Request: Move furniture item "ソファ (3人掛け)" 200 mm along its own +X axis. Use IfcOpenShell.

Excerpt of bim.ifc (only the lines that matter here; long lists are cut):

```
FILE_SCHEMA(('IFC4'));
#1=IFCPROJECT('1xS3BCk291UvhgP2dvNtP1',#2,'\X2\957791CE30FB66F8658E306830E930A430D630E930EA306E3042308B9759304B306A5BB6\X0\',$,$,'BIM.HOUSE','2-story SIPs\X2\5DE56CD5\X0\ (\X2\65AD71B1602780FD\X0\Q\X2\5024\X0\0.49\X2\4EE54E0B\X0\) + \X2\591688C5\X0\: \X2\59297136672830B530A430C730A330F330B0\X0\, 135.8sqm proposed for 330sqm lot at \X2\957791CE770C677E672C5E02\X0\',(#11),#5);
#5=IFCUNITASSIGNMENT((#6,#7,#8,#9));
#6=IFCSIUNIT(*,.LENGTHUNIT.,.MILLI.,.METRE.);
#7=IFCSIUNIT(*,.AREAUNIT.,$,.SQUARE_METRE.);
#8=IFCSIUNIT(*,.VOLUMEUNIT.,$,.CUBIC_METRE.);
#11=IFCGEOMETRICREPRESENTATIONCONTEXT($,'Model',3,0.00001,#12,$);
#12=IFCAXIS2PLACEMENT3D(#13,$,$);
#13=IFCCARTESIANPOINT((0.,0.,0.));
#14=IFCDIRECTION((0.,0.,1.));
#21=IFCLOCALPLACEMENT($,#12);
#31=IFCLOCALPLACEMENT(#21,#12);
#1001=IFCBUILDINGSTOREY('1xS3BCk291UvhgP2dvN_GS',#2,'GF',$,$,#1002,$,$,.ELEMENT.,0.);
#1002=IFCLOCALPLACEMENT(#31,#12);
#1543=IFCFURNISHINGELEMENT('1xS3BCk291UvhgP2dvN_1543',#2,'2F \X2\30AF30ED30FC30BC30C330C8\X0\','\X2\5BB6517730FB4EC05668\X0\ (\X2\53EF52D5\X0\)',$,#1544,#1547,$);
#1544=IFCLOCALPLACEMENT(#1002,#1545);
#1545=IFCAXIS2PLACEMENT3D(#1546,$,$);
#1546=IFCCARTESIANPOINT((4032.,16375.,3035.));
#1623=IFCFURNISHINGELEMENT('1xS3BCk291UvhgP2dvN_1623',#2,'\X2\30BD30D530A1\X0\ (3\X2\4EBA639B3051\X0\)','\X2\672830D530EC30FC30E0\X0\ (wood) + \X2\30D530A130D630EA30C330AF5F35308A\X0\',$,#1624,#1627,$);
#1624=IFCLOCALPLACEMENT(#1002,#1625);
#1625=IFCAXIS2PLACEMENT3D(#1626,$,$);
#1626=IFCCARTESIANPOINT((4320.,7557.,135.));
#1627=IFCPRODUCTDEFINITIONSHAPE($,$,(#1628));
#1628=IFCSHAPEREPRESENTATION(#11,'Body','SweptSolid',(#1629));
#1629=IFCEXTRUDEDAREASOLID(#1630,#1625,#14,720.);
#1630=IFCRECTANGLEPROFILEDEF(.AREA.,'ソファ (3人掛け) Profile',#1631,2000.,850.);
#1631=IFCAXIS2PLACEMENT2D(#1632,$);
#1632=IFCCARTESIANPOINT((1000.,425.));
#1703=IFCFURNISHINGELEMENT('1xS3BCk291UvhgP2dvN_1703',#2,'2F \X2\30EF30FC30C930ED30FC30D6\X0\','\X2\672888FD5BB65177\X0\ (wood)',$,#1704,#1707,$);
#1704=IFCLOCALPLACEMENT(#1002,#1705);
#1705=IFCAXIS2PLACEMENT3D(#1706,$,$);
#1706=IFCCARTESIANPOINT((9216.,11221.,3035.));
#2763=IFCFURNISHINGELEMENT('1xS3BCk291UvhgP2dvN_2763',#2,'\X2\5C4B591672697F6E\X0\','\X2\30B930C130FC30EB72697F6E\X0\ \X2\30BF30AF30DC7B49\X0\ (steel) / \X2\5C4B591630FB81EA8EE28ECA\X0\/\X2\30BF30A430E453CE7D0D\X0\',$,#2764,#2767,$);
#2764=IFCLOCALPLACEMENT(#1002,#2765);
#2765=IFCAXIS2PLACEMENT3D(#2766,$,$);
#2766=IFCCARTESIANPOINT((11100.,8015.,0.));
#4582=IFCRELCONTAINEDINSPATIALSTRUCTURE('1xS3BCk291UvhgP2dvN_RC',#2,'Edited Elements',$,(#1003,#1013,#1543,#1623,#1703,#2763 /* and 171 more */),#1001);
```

```python
import ifcopenshell
import ifcopenshell.api.geometry
import ifcopenshell.util.placement

model = ifcopenshell.open("bim.ifc")

item = model.by_guid("1xS3BCk291UvhgP2dvN_1623")
matrix = ifcopenshell.util.placement.get_local_placement(item.ObjectPlacement)
matrix[:3, 3] += matrix[:3, 0] * 200.0
ifcopenshell.api.geometry.edit_object_placement(model, product=item, matrix=matrix, is_si=False)

print(ifcopenshell.util.placement.get_local_placement(item.ObjectPlacement).round(3) + 0.0)

model.write("bim-out.ifc")
```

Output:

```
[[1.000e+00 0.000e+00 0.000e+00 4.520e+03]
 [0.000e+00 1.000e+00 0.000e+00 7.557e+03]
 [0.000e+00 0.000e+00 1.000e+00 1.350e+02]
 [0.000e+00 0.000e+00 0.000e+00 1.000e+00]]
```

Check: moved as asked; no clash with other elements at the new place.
